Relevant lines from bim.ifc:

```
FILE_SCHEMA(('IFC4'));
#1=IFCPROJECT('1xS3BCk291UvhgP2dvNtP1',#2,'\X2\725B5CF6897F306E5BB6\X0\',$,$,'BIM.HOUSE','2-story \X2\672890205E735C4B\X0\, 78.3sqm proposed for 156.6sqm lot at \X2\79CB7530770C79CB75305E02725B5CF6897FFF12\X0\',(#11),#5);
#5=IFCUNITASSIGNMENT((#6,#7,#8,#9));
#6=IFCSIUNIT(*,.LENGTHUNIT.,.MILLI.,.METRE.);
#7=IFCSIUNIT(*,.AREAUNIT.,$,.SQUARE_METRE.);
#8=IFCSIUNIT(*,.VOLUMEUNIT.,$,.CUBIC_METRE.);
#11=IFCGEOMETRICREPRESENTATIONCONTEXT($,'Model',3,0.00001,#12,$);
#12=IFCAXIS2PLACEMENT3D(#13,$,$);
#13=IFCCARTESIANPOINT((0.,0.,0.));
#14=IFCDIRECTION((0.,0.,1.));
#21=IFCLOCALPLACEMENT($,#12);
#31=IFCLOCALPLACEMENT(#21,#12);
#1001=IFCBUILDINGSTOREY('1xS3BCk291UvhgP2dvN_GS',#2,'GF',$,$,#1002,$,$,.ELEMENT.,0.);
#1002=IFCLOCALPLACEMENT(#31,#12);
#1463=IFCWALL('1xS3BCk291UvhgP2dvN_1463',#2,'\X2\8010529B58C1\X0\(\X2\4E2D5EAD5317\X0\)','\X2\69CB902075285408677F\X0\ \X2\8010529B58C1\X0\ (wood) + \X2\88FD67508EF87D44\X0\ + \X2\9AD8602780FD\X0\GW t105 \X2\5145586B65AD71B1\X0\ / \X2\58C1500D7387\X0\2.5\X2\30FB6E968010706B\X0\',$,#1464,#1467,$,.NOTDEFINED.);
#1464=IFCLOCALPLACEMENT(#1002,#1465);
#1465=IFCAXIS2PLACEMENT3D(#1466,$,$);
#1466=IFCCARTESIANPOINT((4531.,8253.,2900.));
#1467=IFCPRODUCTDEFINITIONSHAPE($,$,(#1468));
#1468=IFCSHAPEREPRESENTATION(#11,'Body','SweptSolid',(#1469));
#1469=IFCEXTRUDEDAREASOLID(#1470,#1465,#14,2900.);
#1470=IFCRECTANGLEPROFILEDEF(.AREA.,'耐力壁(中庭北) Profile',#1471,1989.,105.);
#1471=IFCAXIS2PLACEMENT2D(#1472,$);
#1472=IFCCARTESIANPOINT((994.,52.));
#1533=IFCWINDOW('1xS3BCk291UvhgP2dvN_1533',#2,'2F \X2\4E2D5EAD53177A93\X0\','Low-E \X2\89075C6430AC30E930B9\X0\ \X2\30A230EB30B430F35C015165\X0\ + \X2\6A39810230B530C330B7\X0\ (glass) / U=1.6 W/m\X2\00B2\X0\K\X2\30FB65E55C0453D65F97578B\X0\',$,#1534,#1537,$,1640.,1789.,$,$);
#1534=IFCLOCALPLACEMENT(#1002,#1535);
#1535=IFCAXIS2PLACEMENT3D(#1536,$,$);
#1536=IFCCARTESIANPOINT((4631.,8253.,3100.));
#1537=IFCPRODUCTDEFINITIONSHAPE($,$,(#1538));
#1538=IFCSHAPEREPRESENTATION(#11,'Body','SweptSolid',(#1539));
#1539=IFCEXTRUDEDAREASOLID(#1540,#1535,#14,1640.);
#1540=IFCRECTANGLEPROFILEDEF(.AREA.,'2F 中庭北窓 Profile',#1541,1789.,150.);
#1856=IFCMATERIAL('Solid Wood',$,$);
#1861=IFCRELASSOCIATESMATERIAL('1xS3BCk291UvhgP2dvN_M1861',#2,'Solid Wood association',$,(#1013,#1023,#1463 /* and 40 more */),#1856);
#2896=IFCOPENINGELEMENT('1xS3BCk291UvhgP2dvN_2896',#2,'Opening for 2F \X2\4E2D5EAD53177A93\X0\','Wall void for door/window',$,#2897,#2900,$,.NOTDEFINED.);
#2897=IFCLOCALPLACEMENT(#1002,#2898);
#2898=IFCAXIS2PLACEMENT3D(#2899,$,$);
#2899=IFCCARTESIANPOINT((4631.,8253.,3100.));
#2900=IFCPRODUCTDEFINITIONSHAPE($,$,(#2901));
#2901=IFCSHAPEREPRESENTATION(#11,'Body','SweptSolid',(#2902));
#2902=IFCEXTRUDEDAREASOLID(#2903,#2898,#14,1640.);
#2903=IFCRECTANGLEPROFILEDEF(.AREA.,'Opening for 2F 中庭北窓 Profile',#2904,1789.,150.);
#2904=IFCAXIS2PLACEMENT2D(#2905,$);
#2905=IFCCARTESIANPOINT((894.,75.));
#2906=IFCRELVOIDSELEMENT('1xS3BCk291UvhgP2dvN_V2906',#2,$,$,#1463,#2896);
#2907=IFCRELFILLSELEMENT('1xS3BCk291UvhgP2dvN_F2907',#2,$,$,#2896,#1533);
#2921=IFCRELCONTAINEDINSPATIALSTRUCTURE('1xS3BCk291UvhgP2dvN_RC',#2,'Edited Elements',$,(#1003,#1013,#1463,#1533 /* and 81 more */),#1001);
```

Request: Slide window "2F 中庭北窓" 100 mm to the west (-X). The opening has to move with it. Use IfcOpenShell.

```python
import ifcopenshell
import ifcopenshell.api.geometry
import ifcopenshell.util.placement

model = ifcopenshell.open("bim.ifc")

window = model.by_guid("1xS3BCk291UvhgP2dvN_1533")
opening = window.FillsVoids[0].RelatingOpeningElement
wall = opening.VoidsElements[0].RelatingBuildingElement

wall_matrix = ifcopenshell.util.placement.get_local_placement(wall.ObjectPlacement)
shift = wall_matrix[:3, 0] * -100.0
before = ifcopenshell.util.placement.get_local_placement(window.ObjectPlacement)[:3, 3].copy()

# The window is not placed relative to its opening, so move both.
for product in (opening, window):
    matrix = ifcopenshell.util.placement.get_local_placement(product.ObjectPlacement)
    matrix[:3, 3] += shift
    ifcopenshell.api.geometry.edit_object_placement(model, product=product, matrix=matrix, is_si=False)

after = ifcopenshell.util.placement.get_local_placement(window.ObjectPlacement)[:3, 3]
print("window moved by", (after - before).round(3) + 0.0)

model.write("bim_updated.ifc")
```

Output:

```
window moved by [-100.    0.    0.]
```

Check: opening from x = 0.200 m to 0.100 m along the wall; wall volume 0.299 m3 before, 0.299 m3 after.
